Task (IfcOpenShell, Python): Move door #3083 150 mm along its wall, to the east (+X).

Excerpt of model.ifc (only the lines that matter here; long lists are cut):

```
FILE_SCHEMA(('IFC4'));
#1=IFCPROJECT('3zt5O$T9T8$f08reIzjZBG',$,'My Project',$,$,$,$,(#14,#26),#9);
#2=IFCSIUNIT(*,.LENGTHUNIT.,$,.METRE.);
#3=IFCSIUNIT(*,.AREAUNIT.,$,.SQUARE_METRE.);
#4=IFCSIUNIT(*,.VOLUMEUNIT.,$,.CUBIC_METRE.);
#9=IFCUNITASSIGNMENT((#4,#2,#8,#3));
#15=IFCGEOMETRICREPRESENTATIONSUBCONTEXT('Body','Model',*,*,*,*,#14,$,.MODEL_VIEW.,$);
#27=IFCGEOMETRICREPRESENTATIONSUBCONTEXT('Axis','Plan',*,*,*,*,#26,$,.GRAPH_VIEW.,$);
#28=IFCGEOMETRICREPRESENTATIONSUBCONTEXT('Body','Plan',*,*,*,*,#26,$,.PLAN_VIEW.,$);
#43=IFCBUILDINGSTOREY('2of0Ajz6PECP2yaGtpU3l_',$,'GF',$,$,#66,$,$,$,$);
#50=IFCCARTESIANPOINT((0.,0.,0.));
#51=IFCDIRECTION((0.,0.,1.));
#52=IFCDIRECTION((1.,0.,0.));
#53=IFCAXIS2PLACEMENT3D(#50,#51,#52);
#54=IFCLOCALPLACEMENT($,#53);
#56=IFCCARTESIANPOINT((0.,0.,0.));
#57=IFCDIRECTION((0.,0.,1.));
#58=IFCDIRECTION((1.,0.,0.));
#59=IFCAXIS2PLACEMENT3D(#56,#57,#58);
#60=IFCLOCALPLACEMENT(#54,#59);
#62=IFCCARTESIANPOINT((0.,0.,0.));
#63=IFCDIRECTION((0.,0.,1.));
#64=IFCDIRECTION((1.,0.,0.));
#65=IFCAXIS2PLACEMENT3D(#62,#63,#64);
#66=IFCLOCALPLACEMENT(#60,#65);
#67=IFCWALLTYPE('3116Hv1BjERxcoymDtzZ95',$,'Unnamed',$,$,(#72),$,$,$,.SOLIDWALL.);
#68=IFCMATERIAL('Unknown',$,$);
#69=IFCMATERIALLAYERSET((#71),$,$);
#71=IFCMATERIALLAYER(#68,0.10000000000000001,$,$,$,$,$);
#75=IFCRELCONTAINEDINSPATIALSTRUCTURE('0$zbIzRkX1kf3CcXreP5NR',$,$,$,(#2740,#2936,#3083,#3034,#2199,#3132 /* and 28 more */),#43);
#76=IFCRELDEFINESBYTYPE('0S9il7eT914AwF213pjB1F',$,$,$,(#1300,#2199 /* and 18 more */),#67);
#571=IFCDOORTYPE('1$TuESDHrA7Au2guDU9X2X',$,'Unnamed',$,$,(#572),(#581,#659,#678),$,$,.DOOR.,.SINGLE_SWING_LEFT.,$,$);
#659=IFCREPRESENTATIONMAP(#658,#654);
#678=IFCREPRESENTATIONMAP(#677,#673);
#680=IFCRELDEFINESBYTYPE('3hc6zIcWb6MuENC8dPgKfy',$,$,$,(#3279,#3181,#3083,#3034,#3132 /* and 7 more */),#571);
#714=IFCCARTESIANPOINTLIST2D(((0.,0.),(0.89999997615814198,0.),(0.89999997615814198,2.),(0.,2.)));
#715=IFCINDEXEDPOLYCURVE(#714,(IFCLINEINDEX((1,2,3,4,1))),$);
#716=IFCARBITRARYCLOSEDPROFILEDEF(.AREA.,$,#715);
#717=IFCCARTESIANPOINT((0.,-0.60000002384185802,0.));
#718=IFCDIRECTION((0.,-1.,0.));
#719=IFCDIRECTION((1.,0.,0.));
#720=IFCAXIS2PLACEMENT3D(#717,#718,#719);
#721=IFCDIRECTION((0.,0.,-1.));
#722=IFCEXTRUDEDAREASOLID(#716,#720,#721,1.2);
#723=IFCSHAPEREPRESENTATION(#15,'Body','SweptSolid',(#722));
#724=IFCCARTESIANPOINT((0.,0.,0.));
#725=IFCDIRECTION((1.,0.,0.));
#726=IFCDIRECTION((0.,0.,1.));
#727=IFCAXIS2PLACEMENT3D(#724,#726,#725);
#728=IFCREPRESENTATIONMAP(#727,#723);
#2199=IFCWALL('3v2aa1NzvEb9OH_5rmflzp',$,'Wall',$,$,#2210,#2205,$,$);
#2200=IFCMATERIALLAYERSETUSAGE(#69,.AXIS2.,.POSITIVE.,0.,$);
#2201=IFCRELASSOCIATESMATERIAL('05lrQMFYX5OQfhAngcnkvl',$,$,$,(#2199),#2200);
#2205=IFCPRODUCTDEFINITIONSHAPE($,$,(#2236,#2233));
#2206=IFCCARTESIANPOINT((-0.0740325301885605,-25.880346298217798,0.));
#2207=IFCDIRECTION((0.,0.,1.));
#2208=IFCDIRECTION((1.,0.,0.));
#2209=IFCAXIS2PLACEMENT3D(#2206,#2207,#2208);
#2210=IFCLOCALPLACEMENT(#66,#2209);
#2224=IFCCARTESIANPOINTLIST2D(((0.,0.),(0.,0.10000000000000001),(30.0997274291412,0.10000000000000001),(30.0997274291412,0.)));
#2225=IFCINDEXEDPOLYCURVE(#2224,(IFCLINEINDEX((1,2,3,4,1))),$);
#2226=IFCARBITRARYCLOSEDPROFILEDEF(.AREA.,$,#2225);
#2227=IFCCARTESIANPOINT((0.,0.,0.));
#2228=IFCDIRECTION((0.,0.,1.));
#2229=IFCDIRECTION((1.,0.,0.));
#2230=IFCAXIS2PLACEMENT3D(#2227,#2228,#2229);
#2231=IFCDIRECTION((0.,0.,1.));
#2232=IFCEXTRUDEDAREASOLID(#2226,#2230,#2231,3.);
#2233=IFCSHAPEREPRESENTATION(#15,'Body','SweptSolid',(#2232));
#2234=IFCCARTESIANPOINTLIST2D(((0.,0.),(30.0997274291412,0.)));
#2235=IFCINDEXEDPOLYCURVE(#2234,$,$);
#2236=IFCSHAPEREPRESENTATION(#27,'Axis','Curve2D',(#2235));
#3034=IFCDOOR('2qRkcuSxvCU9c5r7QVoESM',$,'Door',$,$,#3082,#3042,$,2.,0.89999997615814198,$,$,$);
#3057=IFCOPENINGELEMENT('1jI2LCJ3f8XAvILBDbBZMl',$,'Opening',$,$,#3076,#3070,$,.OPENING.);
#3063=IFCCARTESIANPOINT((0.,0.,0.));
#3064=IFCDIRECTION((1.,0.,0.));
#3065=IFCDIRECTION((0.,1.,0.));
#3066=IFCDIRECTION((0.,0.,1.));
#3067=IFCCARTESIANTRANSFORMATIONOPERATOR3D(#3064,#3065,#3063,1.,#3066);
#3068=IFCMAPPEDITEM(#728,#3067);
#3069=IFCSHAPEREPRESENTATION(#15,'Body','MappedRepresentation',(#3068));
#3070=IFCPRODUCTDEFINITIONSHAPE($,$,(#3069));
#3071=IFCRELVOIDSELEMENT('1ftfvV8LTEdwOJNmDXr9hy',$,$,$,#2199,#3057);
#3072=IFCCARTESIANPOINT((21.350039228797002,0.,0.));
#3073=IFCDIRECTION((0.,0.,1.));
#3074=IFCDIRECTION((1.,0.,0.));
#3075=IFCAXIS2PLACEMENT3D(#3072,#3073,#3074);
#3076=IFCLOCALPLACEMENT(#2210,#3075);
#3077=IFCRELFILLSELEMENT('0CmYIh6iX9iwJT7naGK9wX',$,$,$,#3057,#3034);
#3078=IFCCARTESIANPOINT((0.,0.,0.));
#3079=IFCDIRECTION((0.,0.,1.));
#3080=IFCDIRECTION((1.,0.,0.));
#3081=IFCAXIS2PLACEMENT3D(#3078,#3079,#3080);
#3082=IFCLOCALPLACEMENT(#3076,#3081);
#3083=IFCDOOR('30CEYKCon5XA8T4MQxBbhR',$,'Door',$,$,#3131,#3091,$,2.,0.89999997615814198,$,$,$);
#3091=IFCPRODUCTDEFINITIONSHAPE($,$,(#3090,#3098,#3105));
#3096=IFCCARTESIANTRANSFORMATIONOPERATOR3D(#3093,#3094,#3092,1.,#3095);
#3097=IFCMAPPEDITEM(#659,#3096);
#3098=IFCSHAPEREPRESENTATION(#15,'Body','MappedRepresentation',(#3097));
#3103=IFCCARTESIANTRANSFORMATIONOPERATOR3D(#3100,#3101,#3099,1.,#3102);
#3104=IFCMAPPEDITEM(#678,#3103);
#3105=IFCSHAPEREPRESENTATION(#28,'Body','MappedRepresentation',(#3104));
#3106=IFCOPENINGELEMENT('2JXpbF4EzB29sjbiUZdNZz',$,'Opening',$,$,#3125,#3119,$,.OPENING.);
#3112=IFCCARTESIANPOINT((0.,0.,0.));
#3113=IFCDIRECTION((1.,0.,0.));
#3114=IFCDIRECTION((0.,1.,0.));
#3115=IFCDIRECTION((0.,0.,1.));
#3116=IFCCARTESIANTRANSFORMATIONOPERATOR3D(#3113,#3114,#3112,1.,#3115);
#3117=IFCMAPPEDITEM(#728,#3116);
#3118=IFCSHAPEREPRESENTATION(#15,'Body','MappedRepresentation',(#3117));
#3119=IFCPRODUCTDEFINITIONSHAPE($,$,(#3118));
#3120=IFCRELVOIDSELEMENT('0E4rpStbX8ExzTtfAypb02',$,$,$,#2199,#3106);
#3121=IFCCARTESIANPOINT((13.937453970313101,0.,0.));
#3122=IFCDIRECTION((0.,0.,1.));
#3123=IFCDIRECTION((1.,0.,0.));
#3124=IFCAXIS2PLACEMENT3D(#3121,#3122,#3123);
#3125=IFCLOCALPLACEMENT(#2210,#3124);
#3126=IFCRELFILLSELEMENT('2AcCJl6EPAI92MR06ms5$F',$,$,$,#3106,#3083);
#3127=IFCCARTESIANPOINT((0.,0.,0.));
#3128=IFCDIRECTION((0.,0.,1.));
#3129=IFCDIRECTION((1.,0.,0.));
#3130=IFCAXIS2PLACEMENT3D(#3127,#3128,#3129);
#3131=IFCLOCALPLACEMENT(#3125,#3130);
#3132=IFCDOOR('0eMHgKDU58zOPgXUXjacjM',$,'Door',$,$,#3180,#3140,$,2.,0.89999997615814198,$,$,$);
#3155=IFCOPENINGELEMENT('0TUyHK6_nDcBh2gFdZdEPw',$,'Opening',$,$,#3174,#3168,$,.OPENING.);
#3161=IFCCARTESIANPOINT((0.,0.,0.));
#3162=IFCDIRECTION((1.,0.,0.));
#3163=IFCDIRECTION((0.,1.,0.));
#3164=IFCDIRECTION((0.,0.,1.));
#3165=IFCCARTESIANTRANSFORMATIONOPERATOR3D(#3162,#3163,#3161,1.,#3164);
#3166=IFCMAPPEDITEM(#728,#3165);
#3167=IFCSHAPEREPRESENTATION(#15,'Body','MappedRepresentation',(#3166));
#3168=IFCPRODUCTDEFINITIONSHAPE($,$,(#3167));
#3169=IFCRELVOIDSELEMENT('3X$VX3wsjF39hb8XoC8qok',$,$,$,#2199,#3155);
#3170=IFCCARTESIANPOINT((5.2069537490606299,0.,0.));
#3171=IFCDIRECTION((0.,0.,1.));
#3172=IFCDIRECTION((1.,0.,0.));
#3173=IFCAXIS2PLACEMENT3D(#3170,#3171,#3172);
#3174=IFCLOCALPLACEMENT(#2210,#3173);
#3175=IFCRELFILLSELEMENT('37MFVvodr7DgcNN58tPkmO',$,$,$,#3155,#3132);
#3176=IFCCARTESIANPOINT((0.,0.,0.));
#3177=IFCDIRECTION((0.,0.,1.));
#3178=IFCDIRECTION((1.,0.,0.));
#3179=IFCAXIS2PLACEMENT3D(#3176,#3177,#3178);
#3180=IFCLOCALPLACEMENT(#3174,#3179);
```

```python
import ifcopenshell
import ifcopenshell.api.geometry
import ifcopenshell.util.placement
import ifcopenshell.util.unit

model = ifcopenshell.open("model.ifc")
unit_scale = ifcopenshell.util.unit.calculate_unit_scale(model)

door = model.by_guid("30CEYKCon5XA8T4MQxBbhR")
opening = door.FillsVoids[0].RelatingOpeningElement
wall = opening.VoidsElements[0].RelatingBuildingElement

wall_matrix = ifcopenshell.util.placement.get_local_placement(wall.ObjectPlacement)
shift = wall_matrix[:3, 0] * 0.15 / unit_scale
before = ifcopenshell.util.placement.get_local_placement(door.ObjectPlacement)[:3, 3].copy()

# The door is placed relative to its opening, so it follows when the opening moves.
matrix = ifcopenshell.util.placement.get_local_placement(opening.ObjectPlacement)
matrix[:3, 3] += shift
ifcopenshell.api.geometry.edit_object_placement(
    model, product=opening, matrix=matrix, is_si=False, should_transform_children=True
)

after = ifcopenshell.util.placement.get_local_placement(door.ObjectPlacement)[:3, 3]
print("door moved by", (after - before).round(3) + 0.0)

model.write("model_v2.ifc")
```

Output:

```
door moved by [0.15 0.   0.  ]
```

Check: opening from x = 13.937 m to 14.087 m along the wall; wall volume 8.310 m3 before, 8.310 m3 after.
